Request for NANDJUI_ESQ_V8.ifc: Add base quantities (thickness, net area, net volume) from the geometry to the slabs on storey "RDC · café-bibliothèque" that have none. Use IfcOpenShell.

First a look at what the model holds.

```python
import ifcopenshell
import ifcopenshell.util.element
import ifcopenshell.util.unit

model = ifcopenshell.open("NANDJUI_ESQ_V8.ifc")
print(model.schema)
for unit_type in ("LENGTHUNIT", "AREAUNIT", "VOLUMEUNIT"):
    print(unit_type, ifcopenshell.util.unit.calculate_unit_scale(model, unit_type))
storey = next(s for s in model.by_type("IfcBuildingStorey") if s.Name == "RDC · café-bibliothèque")
slabs = [e for e in ifcopenshell.util.element.get_decomposition(storey) if e.is_a("IfcSlab")]
for e in sorted(slabs, key=lambda e: e.id()):
    print(e.id(), e.is_a(), e.Name, list(ifcopenshell.util.element.get_psets(e, qtos_only=True)), sep=" | ")
```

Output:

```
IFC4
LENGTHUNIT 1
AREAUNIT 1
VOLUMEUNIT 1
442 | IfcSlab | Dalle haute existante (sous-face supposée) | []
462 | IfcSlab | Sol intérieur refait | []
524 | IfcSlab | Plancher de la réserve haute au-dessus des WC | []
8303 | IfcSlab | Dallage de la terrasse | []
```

```python
import ifcopenshell
import ifcopenshell.api.pset
import ifcopenshell.geom
import ifcopenshell.util.element
import ifcopenshell.util.shape
import ifcopenshell.util.unit

model = ifcopenshell.open("NANDJUI_ESQ_V8.ifc")
unit_scale = ifcopenshell.util.unit.calculate_unit_scale(model)
area_scale = ifcopenshell.util.unit.calculate_unit_scale(model, "AREAUNIT")
volume_scale = ifcopenshell.util.unit.calculate_unit_scale(model, "VOLUMEUNIT")
settings = ifcopenshell.geom.settings()

storey = next(s for s in model.by_type("IfcBuildingStorey") if s.Name == "RDC · café-bibliothèque")
slabs = [e for e in ifcopenshell.util.element.get_decomposition(storey) if e.is_a("IfcSlab")]

for e in sorted(slabs, key=lambda e: e.id()):
    if ifcopenshell.util.element.get_psets(e, qtos_only=True, should_inherit=False):
        continue
    # Geometry comes back in metres, in the element's own axes.
    shape = ifcopenshell.geom.create_shape(settings, e)
    values = {
        "Width": ifcopenshell.util.shape.get_z(shape.geometry) / unit_scale,
        "NetArea": ifcopenshell.util.shape.get_footprint_area(shape.geometry) / area_scale,
        "NetVolume": ifcopenshell.util.shape.get_volume(shape.geometry) / volume_scale,
    }
    qto = ifcopenshell.api.pset.add_qto(model, product=e, name="Qto_SlabBaseQuantities")
    ifcopenshell.api.pset.edit_qto(model, qto=qto, properties=values)
    print(e.id(), {k: round(v, 3) for k, v in values.items()})

model.write("NANDJUI_ESQ_V8_v2.ifc")
```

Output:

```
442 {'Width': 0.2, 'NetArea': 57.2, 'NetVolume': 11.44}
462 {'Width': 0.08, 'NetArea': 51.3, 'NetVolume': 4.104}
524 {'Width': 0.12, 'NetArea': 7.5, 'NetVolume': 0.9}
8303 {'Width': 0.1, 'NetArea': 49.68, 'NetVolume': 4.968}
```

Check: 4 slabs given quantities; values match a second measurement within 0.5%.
